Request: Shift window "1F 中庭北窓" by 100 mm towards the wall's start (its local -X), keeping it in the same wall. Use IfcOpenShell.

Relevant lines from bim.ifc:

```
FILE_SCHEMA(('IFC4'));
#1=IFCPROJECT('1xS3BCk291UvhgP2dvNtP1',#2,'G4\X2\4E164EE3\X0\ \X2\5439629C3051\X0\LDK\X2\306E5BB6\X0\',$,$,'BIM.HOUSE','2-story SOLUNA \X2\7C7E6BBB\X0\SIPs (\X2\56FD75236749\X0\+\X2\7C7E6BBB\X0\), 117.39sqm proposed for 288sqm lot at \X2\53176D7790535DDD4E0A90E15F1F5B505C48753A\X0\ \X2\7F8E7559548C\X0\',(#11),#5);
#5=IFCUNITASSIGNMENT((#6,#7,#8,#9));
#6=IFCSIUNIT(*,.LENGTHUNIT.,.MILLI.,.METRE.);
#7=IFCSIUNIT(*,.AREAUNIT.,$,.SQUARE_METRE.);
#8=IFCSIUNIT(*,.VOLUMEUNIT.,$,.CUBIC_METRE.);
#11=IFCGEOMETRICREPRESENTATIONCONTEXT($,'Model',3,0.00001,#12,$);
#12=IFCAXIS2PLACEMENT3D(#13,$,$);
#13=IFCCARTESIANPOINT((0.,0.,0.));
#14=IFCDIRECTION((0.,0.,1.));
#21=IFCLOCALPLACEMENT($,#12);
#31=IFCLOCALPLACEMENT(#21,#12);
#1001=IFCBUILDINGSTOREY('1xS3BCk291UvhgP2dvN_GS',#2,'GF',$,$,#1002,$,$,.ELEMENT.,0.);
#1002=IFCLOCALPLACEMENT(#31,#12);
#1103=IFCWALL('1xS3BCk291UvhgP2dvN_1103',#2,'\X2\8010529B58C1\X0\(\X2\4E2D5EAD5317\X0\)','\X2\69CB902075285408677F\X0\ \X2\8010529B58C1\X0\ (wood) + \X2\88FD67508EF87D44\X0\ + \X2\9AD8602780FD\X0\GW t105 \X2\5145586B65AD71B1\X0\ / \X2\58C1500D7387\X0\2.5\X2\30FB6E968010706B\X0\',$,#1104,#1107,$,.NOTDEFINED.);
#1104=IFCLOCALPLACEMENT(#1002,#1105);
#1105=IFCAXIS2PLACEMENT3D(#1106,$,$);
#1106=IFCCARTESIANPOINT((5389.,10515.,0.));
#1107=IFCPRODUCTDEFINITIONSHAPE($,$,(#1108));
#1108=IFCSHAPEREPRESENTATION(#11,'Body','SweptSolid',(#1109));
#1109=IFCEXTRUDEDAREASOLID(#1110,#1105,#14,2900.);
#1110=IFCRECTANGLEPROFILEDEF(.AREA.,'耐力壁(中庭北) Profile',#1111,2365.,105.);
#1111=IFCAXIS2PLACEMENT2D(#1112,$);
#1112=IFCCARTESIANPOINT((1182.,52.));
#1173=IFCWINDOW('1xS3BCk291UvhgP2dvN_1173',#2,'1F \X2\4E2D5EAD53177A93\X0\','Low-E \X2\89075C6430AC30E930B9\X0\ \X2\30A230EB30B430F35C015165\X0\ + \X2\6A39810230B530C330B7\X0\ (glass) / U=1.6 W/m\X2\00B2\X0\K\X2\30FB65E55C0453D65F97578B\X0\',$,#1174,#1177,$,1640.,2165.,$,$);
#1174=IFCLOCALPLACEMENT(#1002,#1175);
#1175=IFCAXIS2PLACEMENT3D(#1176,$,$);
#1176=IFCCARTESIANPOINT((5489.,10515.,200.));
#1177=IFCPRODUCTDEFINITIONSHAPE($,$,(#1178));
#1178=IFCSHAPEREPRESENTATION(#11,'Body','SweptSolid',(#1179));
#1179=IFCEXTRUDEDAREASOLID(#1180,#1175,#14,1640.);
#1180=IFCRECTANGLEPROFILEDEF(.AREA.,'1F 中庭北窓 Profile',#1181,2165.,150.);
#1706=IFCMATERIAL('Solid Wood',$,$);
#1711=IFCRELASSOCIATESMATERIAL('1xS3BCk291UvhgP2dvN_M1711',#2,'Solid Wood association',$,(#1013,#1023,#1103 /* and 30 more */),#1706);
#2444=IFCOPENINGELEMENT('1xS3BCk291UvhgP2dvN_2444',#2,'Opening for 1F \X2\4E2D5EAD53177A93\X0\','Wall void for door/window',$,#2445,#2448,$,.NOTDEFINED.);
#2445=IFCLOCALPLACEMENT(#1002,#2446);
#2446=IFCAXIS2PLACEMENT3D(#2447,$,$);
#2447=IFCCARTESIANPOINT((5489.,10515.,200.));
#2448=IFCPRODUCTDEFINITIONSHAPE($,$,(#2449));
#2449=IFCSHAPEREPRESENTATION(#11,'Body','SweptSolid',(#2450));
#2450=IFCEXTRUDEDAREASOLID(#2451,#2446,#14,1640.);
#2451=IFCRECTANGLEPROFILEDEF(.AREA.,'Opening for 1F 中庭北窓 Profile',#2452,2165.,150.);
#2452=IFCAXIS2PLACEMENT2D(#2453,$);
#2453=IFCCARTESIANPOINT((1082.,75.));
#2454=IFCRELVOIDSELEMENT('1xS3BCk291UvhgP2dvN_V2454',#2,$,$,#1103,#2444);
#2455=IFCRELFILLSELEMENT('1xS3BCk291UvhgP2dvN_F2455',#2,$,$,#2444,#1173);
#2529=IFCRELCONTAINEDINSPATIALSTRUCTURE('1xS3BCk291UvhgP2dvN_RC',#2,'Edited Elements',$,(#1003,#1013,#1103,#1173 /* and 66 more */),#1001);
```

```python
import ifcopenshell
import ifcopenshell.api.geometry
import ifcopenshell.util.placement

model = ifcopenshell.open("bim.ifc")

window = model.by_guid("1xS3BCk291UvhgP2dvN_1173")
opening = window.FillsVoids[0].RelatingOpeningElement
wall = opening.VoidsElements[0].RelatingBuildingElement

wall_matrix = ifcopenshell.util.placement.get_local_placement(wall.ObjectPlacement)
shift = wall_matrix[:3, 0] * -100.0
before = ifcopenshell.util.placement.get_local_placement(window.ObjectPlacement)[:3, 3].copy()

# The window is not placed relative to its opening, so move both.
for product in (opening, window):
    matrix = ifcopenshell.util.placement.get_local_placement(product.ObjectPlacement)
    matrix[:3, 3] += shift
    ifcopenshell.api.geometry.edit_object_placement(model, product=product, matrix=matrix, is_si=False)

after = ifcopenshell.util.placement.get_local_placement(window.ObjectPlacement)[:3, 3]
print("window moved by", (after - before).round(3) + 0.0)

model.write("bim-out.ifc")
```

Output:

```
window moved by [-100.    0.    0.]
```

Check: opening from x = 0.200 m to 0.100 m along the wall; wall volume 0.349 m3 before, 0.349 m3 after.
